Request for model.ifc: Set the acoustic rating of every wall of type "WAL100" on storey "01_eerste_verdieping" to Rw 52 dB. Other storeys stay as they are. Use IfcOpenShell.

First a look at what the model holds.

```python
import ifcopenshell
import ifcopenshell.util.element

model = ifcopenshell.open("model.ifc")
print(model.schema)
storey = next(s for s in model.by_type("IfcBuildingStorey") if s.Name == "01_eerste_verdieping")
walls = [e for e in ifcopenshell.util.element.get_decomposition(storey) if e.is_a("IfcWall")]
seen = {}
for e in walls:
    element_type = ifcopenshell.util.element.get_type(e)
    key = (element_type.Name if element_type != e and element_type else None, ifcopenshell.util.element.get_pset(e, "Pset_WallCommon", "AcousticRating"))
    seen[key] = seen.get(key, 0) + 1
for (name, value), count in sorted(seen.items(), key=str):
    print(count, "x", name, "|", value)
```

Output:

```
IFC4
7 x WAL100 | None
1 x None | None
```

```python
import ifcopenshell
import ifcopenshell.api.pset
import ifcopenshell.util.element

model = ifcopenshell.open("model.ifc")

storey = next(s for s in model.by_type("IfcBuildingStorey") if s.Name == "01_eerste_verdieping")
walls = [e for e in ifcopenshell.util.element.get_decomposition(storey) if e.is_a("IfcWall")]

count = 0
for e in walls:
    element_type = ifcopenshell.util.element.get_type(e)
    if element_type in (None, e) or element_type.Name != "WAL100":
        continue
    # add_pset returns the element's existing set when there is one.
    pset = ifcopenshell.api.pset.add_pset(model, product=e, name="Pset_WallCommon")
    ifcopenshell.api.pset.edit_pset(model, pset=pset, properties={"AcousticRating": "Rw 52 dB"})
    count += 1

print(count, "walls updated")

model.write("model_v2.ifc")
```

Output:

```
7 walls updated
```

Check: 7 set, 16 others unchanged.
